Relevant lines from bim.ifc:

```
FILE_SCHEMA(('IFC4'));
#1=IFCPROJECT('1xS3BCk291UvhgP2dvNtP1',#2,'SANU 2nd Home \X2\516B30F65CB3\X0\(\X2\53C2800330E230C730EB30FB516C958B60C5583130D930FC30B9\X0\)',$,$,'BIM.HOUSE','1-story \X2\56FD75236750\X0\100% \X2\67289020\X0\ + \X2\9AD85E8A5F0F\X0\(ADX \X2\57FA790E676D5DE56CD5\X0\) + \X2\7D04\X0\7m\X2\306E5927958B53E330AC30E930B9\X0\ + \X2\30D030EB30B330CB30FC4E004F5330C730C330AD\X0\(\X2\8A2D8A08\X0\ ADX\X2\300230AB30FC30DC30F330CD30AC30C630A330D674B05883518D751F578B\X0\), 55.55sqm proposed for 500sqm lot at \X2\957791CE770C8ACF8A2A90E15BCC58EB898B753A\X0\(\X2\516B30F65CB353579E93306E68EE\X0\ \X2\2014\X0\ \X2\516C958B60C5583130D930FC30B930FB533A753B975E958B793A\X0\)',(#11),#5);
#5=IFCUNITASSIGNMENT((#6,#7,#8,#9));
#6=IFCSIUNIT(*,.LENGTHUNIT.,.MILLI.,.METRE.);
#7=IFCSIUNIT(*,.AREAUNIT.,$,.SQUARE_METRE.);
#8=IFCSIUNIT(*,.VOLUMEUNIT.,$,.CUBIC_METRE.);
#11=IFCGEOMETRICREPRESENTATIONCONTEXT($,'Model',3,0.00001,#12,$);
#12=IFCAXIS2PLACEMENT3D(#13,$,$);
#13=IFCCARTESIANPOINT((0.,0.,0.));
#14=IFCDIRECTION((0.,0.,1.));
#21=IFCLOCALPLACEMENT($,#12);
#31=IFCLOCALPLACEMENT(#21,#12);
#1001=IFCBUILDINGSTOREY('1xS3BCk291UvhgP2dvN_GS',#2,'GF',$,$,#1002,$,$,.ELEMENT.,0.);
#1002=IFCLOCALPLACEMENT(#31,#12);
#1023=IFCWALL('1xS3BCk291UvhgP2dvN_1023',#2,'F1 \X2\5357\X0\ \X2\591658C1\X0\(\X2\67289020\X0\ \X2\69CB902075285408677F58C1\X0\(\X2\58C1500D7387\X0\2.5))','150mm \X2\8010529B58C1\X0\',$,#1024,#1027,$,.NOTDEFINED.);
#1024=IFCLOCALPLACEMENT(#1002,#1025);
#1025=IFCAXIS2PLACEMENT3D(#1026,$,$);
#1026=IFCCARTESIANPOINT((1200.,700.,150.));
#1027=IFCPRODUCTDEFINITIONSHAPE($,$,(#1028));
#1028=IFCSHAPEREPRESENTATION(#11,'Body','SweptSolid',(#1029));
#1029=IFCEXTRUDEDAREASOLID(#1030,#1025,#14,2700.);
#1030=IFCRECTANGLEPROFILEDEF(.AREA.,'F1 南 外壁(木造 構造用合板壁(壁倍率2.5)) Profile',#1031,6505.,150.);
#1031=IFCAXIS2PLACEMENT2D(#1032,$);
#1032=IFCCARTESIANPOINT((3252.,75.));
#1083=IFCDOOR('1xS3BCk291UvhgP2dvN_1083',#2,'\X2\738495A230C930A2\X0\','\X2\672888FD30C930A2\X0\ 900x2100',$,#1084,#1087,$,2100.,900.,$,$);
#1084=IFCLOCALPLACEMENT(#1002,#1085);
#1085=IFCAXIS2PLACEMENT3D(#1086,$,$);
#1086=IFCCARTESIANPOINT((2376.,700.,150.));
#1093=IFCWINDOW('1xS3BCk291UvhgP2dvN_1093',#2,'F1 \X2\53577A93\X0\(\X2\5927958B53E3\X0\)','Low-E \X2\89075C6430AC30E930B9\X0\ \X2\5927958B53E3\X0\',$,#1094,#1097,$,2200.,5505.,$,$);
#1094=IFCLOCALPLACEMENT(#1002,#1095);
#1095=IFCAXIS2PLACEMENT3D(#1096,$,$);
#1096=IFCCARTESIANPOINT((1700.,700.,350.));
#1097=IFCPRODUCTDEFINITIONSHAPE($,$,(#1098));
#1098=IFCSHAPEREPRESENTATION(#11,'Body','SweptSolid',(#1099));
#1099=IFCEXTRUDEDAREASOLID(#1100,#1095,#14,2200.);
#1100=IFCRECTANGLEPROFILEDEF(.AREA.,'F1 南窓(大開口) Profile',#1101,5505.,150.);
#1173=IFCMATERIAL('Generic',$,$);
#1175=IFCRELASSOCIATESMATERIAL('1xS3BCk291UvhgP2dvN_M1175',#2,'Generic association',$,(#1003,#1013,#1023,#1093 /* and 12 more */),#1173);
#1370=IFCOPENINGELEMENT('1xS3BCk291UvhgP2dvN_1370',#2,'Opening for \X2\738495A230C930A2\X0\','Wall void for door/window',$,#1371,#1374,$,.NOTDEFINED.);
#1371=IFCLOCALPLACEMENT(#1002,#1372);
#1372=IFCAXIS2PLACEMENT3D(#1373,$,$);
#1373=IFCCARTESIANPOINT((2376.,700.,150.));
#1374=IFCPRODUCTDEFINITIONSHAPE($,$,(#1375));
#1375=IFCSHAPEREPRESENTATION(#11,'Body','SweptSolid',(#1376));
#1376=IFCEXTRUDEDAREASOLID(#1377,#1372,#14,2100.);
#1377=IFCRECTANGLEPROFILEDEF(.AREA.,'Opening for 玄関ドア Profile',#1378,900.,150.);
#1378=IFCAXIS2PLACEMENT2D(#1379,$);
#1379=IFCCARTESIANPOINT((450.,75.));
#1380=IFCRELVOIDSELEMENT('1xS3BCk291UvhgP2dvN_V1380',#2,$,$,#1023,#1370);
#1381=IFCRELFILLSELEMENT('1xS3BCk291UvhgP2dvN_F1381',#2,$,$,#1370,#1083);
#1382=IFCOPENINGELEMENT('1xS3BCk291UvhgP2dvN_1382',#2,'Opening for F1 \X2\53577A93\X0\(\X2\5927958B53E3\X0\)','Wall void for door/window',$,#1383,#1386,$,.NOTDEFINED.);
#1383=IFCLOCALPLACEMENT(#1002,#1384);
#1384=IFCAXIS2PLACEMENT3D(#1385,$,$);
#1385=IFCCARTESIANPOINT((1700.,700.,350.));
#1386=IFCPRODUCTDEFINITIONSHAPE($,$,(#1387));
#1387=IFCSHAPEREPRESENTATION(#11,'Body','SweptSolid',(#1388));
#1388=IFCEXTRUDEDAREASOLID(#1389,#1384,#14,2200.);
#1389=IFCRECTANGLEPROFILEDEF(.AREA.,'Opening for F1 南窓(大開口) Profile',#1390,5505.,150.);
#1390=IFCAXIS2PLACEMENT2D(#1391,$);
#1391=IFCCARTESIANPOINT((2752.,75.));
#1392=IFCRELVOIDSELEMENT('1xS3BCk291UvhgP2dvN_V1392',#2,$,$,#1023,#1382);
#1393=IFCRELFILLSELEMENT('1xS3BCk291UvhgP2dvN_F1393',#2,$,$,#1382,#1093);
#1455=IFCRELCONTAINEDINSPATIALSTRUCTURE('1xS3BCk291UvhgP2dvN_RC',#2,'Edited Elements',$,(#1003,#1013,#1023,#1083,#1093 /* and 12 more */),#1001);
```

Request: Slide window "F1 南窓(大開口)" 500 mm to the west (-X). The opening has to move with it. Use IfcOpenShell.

```python
import ifcopenshell
import ifcopenshell.api.geometry
import ifcopenshell.util.placement

model = ifcopenshell.open("bim.ifc")

window = model.by_id(1093)
opening = window.FillsVoids[0].RelatingOpeningElement
wall = opening.VoidsElements[0].RelatingBuildingElement

wall_matrix = ifcopenshell.util.placement.get_local_placement(wall.ObjectPlacement)
shift = wall_matrix[:3, 0] * -500.0
before = ifcopenshell.util.placement.get_local_placement(window.ObjectPlacement)[:3, 3].copy()

# The window is not placed relative to its opening, so move both.
for product in (opening, window):
    matrix = ifcopenshell.util.placement.get_local_placement(product.ObjectPlacement)
    matrix[:3, 3] += shift
    ifcopenshell.api.geometry.edit_object_placement(model, product=product, matrix=matrix, is_si=False)

after = ifcopenshell.util.placement.get_local_placement(window.ObjectPlacement)[:3, 3]
print("window moved by", (after - before).round(3) + 0.0)

model.write("bim_v2.ifc")
```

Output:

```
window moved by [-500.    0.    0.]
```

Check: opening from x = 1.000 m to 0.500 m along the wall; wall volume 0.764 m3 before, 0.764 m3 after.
